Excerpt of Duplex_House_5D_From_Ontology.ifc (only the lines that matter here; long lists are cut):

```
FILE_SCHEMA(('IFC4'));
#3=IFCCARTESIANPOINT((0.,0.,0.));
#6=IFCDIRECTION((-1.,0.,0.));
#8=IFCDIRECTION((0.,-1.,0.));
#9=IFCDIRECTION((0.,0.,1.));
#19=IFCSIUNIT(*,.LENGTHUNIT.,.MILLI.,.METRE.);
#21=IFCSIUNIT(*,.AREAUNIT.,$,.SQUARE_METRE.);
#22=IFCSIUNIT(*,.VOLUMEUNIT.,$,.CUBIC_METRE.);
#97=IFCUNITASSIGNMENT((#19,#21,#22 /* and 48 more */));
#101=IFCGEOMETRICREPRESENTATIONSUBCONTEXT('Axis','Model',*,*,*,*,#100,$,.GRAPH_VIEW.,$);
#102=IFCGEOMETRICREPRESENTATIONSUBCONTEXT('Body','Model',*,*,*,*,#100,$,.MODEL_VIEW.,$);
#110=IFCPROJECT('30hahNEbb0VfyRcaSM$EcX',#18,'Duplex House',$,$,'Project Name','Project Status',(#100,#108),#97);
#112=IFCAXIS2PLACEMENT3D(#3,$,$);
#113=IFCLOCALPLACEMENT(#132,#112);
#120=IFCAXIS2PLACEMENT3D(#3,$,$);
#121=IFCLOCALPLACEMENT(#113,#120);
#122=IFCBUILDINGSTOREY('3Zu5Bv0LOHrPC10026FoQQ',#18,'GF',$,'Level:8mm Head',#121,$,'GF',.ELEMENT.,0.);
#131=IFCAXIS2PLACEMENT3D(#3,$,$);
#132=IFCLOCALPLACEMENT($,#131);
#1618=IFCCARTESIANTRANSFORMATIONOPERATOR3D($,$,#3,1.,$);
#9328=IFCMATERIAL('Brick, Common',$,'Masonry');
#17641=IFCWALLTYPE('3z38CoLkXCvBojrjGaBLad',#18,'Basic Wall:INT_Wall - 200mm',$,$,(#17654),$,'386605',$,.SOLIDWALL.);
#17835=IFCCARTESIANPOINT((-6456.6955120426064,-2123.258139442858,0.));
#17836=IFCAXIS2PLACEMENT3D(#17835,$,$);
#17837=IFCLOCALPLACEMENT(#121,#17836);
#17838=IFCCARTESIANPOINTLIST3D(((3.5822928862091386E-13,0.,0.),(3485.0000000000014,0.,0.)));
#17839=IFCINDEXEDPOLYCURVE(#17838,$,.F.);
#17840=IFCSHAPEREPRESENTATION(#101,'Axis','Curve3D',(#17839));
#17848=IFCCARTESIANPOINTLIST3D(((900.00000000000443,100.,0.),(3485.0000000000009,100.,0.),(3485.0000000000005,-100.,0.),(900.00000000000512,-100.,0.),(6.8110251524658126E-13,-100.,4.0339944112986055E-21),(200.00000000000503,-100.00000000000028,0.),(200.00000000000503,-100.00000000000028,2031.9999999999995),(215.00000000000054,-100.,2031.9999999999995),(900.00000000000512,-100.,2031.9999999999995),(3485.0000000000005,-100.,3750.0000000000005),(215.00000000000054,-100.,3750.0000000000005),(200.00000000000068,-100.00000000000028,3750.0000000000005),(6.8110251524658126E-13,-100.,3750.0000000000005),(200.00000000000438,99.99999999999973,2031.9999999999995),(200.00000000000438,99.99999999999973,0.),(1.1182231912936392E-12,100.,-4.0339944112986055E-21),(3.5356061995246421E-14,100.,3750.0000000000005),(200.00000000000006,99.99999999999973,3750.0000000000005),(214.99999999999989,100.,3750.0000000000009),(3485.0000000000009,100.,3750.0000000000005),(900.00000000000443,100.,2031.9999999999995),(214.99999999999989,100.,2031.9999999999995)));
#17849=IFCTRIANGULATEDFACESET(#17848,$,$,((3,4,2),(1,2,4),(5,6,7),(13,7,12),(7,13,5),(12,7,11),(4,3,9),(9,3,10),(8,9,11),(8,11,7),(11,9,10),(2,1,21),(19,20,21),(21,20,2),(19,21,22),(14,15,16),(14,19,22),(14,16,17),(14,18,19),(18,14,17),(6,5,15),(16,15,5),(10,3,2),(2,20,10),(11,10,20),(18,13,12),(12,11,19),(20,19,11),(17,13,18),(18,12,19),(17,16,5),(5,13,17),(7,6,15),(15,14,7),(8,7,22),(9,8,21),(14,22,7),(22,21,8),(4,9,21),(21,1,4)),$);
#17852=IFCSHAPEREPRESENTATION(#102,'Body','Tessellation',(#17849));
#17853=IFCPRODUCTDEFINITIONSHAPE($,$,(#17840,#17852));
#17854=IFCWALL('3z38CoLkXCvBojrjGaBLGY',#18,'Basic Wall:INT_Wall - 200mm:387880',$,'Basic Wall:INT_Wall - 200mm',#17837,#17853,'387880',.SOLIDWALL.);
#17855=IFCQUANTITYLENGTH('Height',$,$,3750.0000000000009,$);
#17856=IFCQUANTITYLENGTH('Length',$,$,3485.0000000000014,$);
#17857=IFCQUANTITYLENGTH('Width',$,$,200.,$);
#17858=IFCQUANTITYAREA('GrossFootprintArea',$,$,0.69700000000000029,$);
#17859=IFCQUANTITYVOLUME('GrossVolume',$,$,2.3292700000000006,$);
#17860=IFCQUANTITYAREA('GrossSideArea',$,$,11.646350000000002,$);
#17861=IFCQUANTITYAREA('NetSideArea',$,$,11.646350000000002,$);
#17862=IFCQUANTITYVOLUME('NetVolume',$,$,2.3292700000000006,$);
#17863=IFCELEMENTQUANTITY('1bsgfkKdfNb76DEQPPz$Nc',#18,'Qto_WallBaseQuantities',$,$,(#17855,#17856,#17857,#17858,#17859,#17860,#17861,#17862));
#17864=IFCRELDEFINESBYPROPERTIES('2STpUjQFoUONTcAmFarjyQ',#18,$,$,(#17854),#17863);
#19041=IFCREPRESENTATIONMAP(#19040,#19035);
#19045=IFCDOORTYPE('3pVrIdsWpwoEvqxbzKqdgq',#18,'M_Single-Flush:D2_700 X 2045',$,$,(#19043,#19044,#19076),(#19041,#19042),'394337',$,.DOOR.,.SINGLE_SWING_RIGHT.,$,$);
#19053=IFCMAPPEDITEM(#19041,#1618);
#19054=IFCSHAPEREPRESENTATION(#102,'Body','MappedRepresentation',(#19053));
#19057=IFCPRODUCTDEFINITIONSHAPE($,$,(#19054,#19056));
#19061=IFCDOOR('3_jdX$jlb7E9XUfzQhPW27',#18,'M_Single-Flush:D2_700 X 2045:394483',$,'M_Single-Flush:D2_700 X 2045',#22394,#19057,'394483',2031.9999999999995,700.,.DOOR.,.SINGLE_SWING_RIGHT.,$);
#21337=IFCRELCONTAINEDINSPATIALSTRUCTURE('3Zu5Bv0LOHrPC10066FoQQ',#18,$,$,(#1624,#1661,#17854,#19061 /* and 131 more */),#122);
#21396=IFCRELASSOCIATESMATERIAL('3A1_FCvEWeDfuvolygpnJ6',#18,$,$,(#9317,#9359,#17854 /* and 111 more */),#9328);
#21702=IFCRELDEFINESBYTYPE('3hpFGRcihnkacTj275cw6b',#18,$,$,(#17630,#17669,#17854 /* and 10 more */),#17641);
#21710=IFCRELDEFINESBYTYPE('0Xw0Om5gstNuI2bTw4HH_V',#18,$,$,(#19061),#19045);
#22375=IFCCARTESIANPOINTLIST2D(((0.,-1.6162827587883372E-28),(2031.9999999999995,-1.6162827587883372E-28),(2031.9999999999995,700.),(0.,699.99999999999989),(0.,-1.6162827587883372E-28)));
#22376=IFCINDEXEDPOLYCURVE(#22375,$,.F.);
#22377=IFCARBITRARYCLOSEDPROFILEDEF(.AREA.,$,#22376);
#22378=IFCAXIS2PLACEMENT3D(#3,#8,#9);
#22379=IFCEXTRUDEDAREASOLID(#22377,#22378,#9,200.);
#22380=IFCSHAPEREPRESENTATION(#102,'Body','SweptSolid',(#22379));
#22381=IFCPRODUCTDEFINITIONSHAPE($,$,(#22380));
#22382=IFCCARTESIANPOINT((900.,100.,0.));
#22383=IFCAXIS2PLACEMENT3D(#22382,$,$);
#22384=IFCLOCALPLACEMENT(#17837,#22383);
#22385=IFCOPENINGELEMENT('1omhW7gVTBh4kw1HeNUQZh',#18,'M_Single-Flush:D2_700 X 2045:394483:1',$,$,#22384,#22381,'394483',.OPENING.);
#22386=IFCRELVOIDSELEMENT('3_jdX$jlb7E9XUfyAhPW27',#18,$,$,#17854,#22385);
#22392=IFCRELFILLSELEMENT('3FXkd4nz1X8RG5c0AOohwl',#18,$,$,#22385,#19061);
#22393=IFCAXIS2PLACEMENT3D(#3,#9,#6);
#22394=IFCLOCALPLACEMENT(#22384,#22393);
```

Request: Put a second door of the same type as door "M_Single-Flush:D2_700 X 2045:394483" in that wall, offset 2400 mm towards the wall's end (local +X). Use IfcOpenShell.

```python
import ifcopenshell
import ifcopenshell.api.feature
import ifcopenshell.api.geometry
import ifcopenshell.api.pset
import ifcopenshell.api.root
import ifcopenshell.geom
import ifcopenshell.util.element
import ifcopenshell.util.placement
import ifcopenshell.util.shape
import ifcopenshell.util.unit

model = ifcopenshell.open("Duplex_House_5D_From_Ontology.ifc")
unit_scale = ifcopenshell.util.unit.calculate_unit_scale(model)
area_scale = ifcopenshell.util.unit.calculate_unit_scale(model, "AREAUNIT")
volume_scale = ifcopenshell.util.unit.calculate_unit_scale(model, "VOLUMEUNIT")
settings = ifcopenshell.geom.settings()


def volume(element):
    """Net volume in cubic metres, openings subtracted."""
    shape = ifcopenshell.geom.create_shape(settings, element)
    return ifcopenshell.util.shape.get_volume(shape.geometry)


def reuse_history(source, copy):
    """copy_class also copies each property set's owner history, people and application; keep the originals."""
    for rel in copy.IsDefinedBy:
        if rel.is_a("IfcRelDefinesByProperties") and (history := rel.RelatingPropertyDefinition.OwnerHistory):
            rel.RelatingPropertyDefinition.OwnerHistory = source.OwnerHistory
            ifcopenshell.util.element.remove_deep2(model, history)


door = model.by_guid("3_jdX$jlb7E9XUfzQhPW27")
opening = door.FillsVoids[0].RelatingOpeningElement
wall = opening.VoidsElements[0].RelatingBuildingElement
before = volume(wall)
shift = ifcopenshell.util.placement.get_local_placement(wall.ObjectPlacement)[:3, 0] * 2.4 / unit_scale

# copy_class copies the void relationship, type, container and properties, but no geometry.
new_opening = ifcopenshell.api.root.copy_class(model, product=opening)
new_opening.Representation = ifcopenshell.util.element.copy_deep(
    model, opening.Representation, exclude=["IfcGeometricRepresentationContext", "IfcRepresentationMap"]
)
new_opening.Name = "M_Single-Flush:D2_700 X 2045"
new_opening.Tag = None
reuse_history(opening, new_opening)
new_door = ifcopenshell.api.root.copy_class(model, product=door)
new_door.Representation = ifcopenshell.util.element.copy_deep(
    model, door.Representation, exclude=["IfcGeometricRepresentationContext", "IfcRepresentationMap"]
)
new_door.Name = "M_Single-Flush:D2_700 X 2045"
new_door.Tag = None
reuse_history(door, new_door)
ifcopenshell.api.feature.add_filling(model, opening=new_opening, element=new_door)

for old, new in ((opening, new_opening), (door, new_door)):
    matrix = ifcopenshell.util.placement.get_local_placement(old.ObjectPlacement)
    matrix[:3, 3] += shift
    ifcopenshell.api.geometry.edit_object_placement(model, product=new, matrix=matrix, is_si=False)

after = volume(wall)
thickness = 0.2  # wall thickness in metres

# Update the wall's stored quantities.
qto = model.by_id(ifcopenshell.util.element.get_pset(wall, "Qto_WallBaseQuantities", should_inherit=False)["id"])
ifcopenshell.api.pset.edit_qto(model, qto=qto, properties={
    "NetSideArea": after / thickness / area_scale,
    "NetVolume": after / volume_scale,
})

print(f"wall volume {before:.3f} -> {after:.3f} m3")

model.write("Duplex_House_5D_From_Ontology_v2.ifc")
```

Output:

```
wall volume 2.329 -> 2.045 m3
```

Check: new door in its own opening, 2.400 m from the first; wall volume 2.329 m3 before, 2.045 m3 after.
